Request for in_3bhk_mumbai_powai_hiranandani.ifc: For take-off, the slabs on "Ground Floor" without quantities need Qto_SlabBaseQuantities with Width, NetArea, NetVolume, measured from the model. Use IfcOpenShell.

First a look at what the model holds.

```python
import ifcopenshell
import ifcopenshell.util.element
import ifcopenshell.util.unit

model = ifcopenshell.open("in_3bhk_mumbai_powai_hiranandani.ifc")
print(model.schema)
for unit_type in ("LENGTHUNIT", "AREAUNIT", "VOLUMEUNIT"):
    print(unit_type, ifcopenshell.util.unit.calculate_unit_scale(model, unit_type))
storey = next(s for s in model.by_type("IfcBuildingStorey") if s.Name == "Ground Floor")
slabs = [e for e in ifcopenshell.util.element.get_decomposition(storey) if e.is_a("IfcSlab")]
for e in sorted(slabs, key=lambda e: e.id()):
    print(e.id(), e.is_a(), e.Name, list(ifcopenshell.util.element.get_psets(e, qtos_only=True)), sep=" | ")
```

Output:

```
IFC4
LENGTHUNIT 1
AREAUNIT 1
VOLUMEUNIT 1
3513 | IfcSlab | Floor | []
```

```python
import ifcopenshell
import ifcopenshell.api.pset
import ifcopenshell.geom
import ifcopenshell.util.element
import ifcopenshell.util.shape
import ifcopenshell.util.unit

model = ifcopenshell.open("in_3bhk_mumbai_powai_hiranandani.ifc")
unit_scale = ifcopenshell.util.unit.calculate_unit_scale(model)
area_scale = ifcopenshell.util.unit.calculate_unit_scale(model, "AREAUNIT")
volume_scale = ifcopenshell.util.unit.calculate_unit_scale(model, "VOLUMEUNIT")
settings = ifcopenshell.geom.settings()

storey = next(s for s in model.by_type("IfcBuildingStorey") if s.Name == "Ground Floor")
slabs = [e for e in ifcopenshell.util.element.get_decomposition(storey) if e.is_a("IfcSlab")]

for e in sorted(slabs, key=lambda e: e.id()):
    if ifcopenshell.util.element.get_psets(e, qtos_only=True, should_inherit=False):
        continue
    # Geometry comes back in metres, in the element's own axes.
    shape = ifcopenshell.geom.create_shape(settings, e)
    values = {
        "Width": ifcopenshell.util.shape.get_z(shape.geometry) / unit_scale,
        "NetArea": ifcopenshell.util.shape.get_footprint_area(shape.geometry) / area_scale,
        "NetVolume": ifcopenshell.util.shape.get_volume(shape.geometry) / volume_scale,
    }
    qto = ifcopenshell.api.pset.add_qto(model, product=e, name="Qto_SlabBaseQuantities")
    ifcopenshell.api.pset.edit_qto(model, qto=qto, properties=values)
    print(e.id(), {k: round(v, 3) for k, v in values.items()})

model.write("in_3bhk_mumbai_powai_hiranandani-out.ifc")
```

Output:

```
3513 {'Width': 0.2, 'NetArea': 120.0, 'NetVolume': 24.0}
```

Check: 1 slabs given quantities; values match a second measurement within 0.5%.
